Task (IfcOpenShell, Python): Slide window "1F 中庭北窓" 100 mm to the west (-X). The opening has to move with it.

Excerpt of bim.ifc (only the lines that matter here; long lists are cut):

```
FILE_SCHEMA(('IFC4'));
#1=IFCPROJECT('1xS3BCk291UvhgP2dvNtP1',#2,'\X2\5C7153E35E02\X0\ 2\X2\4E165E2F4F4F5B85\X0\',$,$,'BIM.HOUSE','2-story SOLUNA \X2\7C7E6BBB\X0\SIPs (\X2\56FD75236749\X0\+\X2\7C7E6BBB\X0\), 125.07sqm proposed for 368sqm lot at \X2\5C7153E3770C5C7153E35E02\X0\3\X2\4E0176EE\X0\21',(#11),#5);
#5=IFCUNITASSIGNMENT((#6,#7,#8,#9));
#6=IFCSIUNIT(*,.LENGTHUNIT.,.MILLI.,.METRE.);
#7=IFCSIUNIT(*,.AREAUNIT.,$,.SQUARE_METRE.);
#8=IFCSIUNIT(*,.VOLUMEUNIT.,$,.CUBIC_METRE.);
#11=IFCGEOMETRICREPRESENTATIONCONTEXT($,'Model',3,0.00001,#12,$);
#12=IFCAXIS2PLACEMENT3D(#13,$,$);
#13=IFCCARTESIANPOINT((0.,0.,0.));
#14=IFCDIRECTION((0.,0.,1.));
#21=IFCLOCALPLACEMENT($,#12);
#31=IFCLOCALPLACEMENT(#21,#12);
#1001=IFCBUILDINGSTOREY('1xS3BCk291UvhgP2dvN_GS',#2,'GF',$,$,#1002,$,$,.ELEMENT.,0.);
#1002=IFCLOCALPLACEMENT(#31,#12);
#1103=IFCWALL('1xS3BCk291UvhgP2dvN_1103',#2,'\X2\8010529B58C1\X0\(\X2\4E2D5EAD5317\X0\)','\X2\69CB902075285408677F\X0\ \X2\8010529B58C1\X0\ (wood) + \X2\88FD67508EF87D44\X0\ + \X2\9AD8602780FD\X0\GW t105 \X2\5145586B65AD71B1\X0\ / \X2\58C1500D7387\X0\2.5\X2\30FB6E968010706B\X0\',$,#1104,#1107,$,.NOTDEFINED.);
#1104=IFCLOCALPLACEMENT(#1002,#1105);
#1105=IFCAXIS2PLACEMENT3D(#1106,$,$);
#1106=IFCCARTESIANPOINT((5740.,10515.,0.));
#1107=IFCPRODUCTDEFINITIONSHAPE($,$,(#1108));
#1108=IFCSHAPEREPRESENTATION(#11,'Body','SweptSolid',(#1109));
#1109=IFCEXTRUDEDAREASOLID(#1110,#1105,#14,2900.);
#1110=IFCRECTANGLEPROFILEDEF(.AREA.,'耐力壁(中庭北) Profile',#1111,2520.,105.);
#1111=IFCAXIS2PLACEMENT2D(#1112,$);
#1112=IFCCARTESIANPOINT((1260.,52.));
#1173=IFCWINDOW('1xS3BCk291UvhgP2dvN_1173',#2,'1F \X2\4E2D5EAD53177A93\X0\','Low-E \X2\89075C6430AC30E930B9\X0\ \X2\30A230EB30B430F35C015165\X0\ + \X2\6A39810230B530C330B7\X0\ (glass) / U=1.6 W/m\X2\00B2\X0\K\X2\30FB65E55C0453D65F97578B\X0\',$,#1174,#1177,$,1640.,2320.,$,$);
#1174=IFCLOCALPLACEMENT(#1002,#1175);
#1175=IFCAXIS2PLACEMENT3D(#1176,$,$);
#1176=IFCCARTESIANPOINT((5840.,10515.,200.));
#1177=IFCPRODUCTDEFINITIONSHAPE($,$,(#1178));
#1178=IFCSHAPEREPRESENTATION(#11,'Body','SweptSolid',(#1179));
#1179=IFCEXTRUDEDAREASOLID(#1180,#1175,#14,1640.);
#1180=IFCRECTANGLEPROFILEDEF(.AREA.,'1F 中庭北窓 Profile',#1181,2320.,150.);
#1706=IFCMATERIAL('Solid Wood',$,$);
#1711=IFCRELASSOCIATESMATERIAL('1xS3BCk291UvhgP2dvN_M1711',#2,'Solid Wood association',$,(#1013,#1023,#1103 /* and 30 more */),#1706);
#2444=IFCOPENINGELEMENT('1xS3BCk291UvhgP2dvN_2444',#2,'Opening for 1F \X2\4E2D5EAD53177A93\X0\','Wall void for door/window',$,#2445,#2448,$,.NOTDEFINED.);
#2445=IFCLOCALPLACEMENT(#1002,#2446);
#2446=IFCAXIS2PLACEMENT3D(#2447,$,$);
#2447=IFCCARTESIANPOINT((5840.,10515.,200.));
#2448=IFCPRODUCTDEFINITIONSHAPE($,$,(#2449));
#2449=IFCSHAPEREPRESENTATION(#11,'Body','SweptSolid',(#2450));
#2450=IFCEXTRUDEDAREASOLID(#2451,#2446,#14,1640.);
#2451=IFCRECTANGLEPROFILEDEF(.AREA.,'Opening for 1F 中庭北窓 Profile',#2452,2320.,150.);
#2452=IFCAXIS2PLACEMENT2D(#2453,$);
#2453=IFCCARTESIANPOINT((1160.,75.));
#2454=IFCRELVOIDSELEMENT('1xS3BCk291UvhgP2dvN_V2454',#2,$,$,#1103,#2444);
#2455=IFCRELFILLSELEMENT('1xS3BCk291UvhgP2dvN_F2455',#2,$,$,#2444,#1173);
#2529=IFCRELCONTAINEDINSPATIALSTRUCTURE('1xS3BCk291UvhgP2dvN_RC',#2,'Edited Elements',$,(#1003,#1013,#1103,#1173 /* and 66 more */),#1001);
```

```python
import ifcopenshell
import ifcopenshell.api.geometry
import ifcopenshell.util.placement

model = ifcopenshell.open("bim.ifc")

window = model.by_id(1173)
opening = window.FillsVoids[0].RelatingOpeningElement
wall = opening.VoidsElements[0].RelatingBuildingElement

wall_matrix = ifcopenshell.util.placement.get_local_placement(wall.ObjectPlacement)
shift = wall_matrix[:3, 0] * -100.0
before = ifcopenshell.util.placement.get_local_placement(window.ObjectPlacement)[:3, 3].copy()

# The window is not placed relative to its opening, so move both.
for product in (opening, window):
    matrix = ifcopenshell.util.placement.get_local_placement(product.ObjectPlacement)
    matrix[:3, 3] += shift
    ifcopenshell.api.geometry.edit_object_placement(model, product=product, matrix=matrix, is_si=False)

after = ifcopenshell.util.placement.get_local_placement(window.ObjectPlacement)[:3, 3]
print("window moved by", (after - before).round(3) + 0.0)

model.write("bim_edited.ifc")
```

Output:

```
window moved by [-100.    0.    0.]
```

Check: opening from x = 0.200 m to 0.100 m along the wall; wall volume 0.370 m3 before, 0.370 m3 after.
